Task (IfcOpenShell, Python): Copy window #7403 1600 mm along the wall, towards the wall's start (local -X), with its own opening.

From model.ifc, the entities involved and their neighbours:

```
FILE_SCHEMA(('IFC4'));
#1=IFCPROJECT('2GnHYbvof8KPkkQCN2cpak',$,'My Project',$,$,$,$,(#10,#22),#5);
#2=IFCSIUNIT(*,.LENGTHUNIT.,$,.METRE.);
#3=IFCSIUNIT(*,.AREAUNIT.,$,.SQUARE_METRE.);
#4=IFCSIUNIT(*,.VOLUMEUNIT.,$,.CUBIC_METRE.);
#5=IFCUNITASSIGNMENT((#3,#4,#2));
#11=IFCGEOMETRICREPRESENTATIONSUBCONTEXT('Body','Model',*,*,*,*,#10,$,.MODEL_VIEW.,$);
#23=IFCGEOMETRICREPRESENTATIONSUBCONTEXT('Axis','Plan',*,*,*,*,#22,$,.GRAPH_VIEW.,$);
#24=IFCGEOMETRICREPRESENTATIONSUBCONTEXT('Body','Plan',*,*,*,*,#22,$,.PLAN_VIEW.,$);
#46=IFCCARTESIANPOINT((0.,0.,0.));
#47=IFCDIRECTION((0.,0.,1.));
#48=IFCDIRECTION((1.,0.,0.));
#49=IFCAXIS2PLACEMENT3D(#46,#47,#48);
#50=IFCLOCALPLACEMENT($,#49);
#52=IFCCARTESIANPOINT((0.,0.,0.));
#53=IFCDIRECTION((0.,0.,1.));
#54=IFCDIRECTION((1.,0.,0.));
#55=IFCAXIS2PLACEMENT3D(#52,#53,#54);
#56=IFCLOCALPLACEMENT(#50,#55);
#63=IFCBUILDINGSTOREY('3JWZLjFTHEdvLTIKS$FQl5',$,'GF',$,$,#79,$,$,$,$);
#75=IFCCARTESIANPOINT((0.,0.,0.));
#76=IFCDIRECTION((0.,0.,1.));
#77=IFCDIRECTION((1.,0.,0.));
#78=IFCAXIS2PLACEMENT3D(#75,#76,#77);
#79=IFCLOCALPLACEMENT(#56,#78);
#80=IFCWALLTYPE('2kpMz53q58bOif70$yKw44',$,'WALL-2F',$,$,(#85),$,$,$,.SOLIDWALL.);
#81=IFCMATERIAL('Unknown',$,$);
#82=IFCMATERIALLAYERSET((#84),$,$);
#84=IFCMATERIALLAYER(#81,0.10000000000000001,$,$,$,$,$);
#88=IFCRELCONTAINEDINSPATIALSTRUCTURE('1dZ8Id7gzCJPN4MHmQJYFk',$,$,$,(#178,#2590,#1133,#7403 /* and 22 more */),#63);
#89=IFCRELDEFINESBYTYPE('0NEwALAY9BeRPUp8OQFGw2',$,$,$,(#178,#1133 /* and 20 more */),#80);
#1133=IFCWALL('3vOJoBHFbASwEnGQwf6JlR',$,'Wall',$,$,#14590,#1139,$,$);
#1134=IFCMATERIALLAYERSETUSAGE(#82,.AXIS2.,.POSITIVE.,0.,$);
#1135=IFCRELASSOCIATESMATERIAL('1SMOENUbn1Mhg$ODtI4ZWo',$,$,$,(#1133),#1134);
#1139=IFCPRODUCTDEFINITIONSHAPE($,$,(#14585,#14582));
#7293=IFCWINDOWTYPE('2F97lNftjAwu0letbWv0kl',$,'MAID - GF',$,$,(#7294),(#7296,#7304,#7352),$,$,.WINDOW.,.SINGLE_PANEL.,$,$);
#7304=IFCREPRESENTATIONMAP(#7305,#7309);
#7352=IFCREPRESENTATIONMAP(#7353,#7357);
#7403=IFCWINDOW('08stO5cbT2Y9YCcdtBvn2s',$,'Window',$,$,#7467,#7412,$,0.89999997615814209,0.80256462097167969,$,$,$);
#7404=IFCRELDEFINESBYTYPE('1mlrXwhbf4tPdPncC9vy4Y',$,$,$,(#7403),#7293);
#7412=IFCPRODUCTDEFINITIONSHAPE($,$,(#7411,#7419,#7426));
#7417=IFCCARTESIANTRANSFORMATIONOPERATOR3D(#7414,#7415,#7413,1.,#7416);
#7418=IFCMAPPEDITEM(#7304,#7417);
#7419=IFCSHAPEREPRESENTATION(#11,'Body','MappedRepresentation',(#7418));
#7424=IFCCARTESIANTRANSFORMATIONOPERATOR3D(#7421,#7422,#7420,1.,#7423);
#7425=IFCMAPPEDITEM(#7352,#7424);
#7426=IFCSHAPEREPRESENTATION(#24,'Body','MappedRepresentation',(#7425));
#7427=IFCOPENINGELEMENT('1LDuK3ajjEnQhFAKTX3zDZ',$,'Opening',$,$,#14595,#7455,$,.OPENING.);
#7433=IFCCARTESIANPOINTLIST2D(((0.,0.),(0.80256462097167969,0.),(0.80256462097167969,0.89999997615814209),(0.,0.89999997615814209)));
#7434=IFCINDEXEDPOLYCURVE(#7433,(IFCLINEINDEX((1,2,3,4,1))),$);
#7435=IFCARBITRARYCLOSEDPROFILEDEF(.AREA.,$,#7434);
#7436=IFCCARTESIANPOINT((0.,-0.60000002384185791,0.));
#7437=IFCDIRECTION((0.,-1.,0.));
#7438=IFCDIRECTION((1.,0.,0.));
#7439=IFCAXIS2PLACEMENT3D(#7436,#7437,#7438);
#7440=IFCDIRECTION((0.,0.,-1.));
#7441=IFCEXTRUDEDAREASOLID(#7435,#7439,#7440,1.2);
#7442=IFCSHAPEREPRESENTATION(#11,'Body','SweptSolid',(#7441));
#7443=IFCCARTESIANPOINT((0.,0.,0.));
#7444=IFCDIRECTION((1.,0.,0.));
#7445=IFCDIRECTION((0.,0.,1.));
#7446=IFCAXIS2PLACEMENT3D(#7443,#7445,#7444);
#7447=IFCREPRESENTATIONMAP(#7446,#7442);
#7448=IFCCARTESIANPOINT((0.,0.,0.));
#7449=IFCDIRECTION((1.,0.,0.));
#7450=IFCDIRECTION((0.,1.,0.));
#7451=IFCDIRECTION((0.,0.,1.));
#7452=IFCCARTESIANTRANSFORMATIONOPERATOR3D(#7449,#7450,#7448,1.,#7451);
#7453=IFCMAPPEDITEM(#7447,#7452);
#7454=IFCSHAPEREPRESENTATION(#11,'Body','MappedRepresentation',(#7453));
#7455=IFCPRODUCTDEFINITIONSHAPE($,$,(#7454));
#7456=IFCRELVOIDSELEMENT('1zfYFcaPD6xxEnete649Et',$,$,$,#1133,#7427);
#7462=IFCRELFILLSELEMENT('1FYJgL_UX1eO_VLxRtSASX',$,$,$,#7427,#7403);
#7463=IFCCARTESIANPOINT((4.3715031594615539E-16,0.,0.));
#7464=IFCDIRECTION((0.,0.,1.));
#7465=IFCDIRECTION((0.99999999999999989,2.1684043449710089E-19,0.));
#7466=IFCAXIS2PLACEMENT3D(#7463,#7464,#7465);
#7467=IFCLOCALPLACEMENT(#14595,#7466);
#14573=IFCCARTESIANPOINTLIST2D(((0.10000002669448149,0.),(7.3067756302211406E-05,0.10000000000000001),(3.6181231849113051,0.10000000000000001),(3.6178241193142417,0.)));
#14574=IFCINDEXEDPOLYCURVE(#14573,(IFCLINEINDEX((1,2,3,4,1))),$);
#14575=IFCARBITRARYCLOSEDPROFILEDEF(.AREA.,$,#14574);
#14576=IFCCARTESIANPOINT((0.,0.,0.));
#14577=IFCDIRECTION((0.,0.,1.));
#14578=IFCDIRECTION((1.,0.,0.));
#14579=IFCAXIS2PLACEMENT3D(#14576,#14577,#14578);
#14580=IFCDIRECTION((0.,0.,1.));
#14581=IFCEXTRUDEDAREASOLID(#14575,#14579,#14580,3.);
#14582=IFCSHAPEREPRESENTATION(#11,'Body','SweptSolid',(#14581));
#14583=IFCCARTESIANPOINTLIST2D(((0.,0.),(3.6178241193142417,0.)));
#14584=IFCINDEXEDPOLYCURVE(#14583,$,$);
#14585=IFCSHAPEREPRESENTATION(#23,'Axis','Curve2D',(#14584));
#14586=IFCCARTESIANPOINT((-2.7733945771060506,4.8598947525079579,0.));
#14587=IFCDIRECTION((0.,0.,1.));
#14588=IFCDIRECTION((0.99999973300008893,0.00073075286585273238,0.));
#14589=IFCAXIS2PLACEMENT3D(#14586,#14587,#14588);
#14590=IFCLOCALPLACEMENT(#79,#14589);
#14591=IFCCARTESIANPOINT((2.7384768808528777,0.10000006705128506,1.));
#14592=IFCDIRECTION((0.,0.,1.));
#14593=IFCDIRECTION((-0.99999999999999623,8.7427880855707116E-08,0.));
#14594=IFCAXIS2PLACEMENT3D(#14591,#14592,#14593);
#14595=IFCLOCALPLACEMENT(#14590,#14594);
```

```python
import ifcopenshell
import ifcopenshell.api.feature
import ifcopenshell.api.geometry
import ifcopenshell.api.root
import ifcopenshell.geom
import ifcopenshell.util.element
import ifcopenshell.util.placement
import ifcopenshell.util.shape

model = ifcopenshell.open("model.ifc")
settings = ifcopenshell.geom.settings()


def volume(element):
    """Net volume in cubic metres, openings subtracted."""
    shape = ifcopenshell.geom.create_shape(settings, element)
    return ifcopenshell.util.shape.get_volume(shape.geometry)


window = model.by_guid("08stO5cbT2Y9YCcdtBvn2s")
opening = window.FillsVoids[0].RelatingOpeningElement
wall = opening.VoidsElements[0].RelatingBuildingElement
before = volume(wall)
shift = ifcopenshell.util.placement.get_local_placement(wall.ObjectPlacement)[:3, 0] * -1.6

# copy_class copies the void relationship, type, container and properties, but no geometry.
new_opening = ifcopenshell.api.root.copy_class(model, product=opening)
new_opening.Representation = ifcopenshell.util.element.copy_deep(
    model, opening.Representation, exclude=["IfcGeometricRepresentationContext", "IfcRepresentationMap"]
)
new_window = ifcopenshell.api.root.copy_class(model, product=window)
new_window.Representation = ifcopenshell.util.element.copy_deep(
    model, window.Representation, exclude=["IfcGeometricRepresentationContext", "IfcRepresentationMap"]
)
ifcopenshell.api.feature.add_filling(model, opening=new_opening, element=new_window)

for old, new in ((opening, new_opening), (window, new_window)):
    matrix = ifcopenshell.util.placement.get_local_placement(old.ObjectPlacement)
    matrix[:3, 3] += shift
    ifcopenshell.api.geometry.edit_object_placement(model, product=new, matrix=matrix, is_si=False)

after = volume(wall)

print(f"wall volume {before:.3f} -> {after:.3f} m3")

model.write("model_updated.ifc")
```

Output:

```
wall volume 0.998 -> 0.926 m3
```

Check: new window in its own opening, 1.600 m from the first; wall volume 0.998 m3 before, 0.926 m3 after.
